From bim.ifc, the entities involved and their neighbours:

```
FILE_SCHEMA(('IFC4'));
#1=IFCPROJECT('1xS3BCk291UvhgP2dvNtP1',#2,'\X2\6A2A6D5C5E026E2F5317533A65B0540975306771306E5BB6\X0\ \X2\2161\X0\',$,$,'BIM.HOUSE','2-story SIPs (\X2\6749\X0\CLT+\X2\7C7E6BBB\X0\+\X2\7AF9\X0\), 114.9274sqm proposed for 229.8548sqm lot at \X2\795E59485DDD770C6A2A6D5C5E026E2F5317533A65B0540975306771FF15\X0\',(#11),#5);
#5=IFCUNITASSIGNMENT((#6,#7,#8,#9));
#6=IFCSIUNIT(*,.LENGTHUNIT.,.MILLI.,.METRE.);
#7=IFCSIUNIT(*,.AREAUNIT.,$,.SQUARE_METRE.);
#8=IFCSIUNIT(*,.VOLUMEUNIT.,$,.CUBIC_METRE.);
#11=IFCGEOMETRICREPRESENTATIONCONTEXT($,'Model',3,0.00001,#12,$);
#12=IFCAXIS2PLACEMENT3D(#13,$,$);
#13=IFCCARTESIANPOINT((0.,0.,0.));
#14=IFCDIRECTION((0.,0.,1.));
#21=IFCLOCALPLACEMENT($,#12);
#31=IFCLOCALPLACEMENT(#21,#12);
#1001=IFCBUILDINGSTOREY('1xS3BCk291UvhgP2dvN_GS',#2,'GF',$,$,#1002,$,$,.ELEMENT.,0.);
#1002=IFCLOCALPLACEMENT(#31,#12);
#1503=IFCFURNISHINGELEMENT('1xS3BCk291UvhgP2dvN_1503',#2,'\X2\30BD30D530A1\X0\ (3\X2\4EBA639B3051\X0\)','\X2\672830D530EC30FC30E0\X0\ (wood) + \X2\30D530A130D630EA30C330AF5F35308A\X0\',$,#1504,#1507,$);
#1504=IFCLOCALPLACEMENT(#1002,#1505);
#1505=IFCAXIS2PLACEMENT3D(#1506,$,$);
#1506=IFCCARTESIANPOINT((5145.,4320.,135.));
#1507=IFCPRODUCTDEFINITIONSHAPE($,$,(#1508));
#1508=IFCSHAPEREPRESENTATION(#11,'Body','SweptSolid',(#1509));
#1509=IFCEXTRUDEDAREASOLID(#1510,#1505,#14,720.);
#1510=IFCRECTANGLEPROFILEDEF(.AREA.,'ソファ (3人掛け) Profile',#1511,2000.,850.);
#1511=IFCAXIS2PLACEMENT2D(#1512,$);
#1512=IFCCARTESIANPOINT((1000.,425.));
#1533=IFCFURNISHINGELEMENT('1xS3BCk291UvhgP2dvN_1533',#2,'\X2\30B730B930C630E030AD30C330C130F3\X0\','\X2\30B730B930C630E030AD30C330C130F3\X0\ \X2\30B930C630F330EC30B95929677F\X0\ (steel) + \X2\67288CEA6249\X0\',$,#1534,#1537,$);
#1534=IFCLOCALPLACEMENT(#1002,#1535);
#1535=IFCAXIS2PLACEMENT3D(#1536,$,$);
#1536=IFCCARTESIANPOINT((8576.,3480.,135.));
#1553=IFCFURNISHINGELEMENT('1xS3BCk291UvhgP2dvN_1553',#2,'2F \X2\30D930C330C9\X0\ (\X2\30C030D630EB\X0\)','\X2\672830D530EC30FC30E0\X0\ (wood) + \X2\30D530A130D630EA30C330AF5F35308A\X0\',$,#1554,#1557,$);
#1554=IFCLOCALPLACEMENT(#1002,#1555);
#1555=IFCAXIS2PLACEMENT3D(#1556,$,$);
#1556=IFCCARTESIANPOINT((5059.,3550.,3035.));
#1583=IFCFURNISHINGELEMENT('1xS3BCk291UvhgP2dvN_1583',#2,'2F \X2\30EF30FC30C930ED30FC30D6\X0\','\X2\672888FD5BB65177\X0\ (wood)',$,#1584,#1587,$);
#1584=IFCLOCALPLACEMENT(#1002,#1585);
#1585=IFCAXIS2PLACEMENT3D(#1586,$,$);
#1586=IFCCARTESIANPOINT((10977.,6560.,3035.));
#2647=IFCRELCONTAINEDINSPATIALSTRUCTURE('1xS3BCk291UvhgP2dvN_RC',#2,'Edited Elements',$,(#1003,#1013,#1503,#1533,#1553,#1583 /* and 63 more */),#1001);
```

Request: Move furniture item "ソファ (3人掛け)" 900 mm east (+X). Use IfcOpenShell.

```python
import ifcopenshell
import ifcopenshell.api.geometry
import ifcopenshell.util.placement
import ifcopenshell.util.unit

model = ifcopenshell.open("bim.ifc")
unit_scale = ifcopenshell.util.unit.calculate_unit_scale(model)

item = model.by_guid("1xS3BCk291UvhgP2dvN_1503")
matrix = ifcopenshell.util.placement.get_local_placement(item.ObjectPlacement)
matrix[0, 3] += 0.9 / unit_scale
ifcopenshell.api.geometry.edit_object_placement(model, product=item, matrix=matrix, is_si=False)

print(ifcopenshell.util.placement.get_local_placement(item.ObjectPlacement).round(3) + 0.0)

model.write("bim_v2.ifc")
```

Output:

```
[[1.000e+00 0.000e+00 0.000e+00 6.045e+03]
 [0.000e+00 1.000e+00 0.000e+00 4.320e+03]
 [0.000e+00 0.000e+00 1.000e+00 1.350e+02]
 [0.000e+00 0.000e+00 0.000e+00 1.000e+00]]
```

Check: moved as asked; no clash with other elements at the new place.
